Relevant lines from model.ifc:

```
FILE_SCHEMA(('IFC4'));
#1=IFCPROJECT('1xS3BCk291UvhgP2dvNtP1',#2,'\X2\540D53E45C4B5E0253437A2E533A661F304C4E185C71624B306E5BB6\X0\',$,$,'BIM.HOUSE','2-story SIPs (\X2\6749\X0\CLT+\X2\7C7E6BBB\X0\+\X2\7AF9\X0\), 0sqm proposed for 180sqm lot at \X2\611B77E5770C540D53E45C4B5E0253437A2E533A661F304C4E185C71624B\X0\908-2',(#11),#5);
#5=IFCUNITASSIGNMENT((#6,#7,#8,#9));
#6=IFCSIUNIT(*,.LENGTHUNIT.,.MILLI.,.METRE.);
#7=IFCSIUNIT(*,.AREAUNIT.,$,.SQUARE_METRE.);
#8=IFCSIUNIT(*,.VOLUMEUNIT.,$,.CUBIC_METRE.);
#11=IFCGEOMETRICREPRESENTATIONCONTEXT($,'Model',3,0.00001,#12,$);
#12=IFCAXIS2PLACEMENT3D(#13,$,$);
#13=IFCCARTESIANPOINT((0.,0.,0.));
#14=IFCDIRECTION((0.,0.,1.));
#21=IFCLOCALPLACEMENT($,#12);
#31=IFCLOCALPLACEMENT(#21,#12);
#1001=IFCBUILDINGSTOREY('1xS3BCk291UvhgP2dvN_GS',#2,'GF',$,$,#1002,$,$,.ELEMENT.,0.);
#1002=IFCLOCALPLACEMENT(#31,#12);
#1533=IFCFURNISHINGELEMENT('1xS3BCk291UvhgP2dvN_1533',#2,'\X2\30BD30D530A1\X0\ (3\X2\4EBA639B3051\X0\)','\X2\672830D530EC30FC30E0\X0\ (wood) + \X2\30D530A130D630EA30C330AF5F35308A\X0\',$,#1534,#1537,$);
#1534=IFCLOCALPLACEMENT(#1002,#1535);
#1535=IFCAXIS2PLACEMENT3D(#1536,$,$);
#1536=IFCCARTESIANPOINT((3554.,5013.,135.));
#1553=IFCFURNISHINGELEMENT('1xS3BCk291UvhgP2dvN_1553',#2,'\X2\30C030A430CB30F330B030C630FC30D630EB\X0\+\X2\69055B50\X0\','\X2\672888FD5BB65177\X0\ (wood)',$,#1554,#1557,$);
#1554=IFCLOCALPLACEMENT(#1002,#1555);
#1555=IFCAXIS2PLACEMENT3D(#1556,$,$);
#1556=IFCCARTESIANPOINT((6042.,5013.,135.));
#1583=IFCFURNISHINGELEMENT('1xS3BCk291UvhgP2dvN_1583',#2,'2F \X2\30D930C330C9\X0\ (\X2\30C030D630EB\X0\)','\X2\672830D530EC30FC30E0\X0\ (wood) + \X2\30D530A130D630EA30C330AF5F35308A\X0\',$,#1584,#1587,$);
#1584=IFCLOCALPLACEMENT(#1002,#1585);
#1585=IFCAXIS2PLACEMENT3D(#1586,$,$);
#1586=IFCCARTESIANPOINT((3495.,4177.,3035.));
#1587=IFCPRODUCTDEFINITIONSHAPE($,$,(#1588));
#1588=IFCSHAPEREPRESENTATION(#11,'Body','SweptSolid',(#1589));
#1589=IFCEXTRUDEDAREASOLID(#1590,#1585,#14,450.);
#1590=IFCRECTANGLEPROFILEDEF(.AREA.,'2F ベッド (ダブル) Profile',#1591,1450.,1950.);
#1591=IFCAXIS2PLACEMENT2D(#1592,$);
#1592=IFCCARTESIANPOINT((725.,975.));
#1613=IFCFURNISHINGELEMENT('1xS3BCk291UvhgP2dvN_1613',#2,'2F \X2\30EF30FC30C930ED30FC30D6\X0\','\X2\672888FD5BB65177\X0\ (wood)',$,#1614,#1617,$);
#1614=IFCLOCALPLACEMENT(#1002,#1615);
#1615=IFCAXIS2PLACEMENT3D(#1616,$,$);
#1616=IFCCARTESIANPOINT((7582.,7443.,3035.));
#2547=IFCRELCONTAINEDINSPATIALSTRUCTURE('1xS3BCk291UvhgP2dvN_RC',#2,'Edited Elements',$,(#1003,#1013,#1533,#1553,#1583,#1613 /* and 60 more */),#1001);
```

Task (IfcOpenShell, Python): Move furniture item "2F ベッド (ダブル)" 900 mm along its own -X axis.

```python
import ifcopenshell
import ifcopenshell.api.geometry
import ifcopenshell.util.placement

model = ifcopenshell.open("model.ifc")

item = model.by_guid("1xS3BCk291UvhgP2dvN_1583")
matrix = ifcopenshell.util.placement.get_local_placement(item.ObjectPlacement)
matrix[:3, 3] -= matrix[:3, 0] * 900.0
ifcopenshell.api.geometry.edit_object_placement(model, product=item, matrix=matrix, is_si=False)

print(ifcopenshell.util.placement.get_local_placement(item.ObjectPlacement).round(3) + 0.0)

model.write("model_rev.ifc")
```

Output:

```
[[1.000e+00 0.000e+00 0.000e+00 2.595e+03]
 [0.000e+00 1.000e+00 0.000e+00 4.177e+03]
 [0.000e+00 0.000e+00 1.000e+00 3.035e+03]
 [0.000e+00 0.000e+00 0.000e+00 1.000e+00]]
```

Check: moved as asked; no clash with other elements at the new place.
